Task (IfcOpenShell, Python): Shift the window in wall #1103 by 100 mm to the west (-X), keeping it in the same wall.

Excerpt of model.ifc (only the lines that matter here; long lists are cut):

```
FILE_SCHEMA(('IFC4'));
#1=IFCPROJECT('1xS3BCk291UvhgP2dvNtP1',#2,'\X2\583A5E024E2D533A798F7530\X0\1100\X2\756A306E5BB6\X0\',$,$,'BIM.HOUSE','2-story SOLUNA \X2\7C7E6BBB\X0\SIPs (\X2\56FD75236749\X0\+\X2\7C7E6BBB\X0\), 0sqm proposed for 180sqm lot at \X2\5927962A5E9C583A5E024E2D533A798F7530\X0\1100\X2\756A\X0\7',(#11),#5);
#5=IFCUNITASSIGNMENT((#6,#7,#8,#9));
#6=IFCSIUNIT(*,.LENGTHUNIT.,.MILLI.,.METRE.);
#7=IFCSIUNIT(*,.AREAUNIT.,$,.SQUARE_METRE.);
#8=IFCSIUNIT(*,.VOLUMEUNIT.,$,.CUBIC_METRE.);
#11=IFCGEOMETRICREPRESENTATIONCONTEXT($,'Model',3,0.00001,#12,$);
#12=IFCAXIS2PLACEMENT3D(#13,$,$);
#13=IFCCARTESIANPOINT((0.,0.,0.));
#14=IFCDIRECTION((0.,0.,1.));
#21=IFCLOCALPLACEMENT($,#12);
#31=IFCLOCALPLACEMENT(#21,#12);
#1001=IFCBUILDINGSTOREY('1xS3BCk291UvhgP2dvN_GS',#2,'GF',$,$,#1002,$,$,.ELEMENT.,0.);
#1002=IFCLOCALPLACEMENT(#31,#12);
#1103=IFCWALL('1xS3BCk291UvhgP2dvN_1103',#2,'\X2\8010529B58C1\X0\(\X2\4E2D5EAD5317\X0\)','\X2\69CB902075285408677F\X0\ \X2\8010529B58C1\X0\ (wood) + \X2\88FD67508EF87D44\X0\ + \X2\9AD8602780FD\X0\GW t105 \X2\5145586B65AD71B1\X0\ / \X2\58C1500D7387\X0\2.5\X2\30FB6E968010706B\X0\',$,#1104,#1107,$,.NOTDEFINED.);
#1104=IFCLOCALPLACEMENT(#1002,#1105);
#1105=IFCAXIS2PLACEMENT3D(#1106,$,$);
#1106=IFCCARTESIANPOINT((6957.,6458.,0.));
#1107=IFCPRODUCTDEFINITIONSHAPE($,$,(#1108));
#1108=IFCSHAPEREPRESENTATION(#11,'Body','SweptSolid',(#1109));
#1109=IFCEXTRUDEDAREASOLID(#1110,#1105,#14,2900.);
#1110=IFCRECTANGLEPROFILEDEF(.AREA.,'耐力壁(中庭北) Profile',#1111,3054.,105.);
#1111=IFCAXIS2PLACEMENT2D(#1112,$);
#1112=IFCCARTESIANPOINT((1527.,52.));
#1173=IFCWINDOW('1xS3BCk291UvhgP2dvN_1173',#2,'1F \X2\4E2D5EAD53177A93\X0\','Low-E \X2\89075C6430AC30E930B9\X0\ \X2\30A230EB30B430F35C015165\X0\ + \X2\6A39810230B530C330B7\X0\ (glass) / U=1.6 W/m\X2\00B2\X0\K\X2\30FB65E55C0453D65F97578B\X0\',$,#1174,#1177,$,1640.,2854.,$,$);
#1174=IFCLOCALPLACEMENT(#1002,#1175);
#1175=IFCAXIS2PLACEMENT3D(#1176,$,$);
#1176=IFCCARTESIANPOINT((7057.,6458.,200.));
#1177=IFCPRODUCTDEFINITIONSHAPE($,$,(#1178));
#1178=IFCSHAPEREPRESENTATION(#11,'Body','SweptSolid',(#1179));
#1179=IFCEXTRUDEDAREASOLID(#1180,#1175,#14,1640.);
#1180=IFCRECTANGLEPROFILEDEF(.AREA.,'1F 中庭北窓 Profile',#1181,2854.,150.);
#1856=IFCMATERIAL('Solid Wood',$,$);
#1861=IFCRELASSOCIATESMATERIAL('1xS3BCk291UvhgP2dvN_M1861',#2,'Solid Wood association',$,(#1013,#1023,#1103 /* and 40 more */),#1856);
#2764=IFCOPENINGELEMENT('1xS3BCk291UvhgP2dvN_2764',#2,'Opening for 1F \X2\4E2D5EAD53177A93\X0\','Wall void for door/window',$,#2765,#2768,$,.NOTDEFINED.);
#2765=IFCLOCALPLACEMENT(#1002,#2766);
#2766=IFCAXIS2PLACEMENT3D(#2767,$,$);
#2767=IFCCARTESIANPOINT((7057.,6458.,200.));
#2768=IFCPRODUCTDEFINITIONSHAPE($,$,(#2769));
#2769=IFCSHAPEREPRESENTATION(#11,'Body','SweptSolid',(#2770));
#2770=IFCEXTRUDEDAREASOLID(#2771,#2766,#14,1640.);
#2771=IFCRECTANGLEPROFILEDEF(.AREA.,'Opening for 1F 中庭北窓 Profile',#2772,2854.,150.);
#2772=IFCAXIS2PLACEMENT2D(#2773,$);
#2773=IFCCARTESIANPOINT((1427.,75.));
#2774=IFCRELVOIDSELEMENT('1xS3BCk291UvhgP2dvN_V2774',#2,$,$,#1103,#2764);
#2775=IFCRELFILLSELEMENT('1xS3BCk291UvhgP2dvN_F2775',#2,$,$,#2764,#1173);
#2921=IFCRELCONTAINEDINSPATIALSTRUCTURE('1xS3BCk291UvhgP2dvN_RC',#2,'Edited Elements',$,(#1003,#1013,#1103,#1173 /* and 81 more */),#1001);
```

```python
import ifcopenshell
import ifcopenshell.api.geometry
import ifcopenshell.util.placement
import ifcopenshell.util.unit

model = ifcopenshell.open("model.ifc")
unit_scale = ifcopenshell.util.unit.calculate_unit_scale(model)

window = model.by_guid("1xS3BCk291UvhgP2dvN_1173")
opening = window.FillsVoids[0].RelatingOpeningElement
wall = opening.VoidsElements[0].RelatingBuildingElement

wall_matrix = ifcopenshell.util.placement.get_local_placement(wall.ObjectPlacement)
shift = wall_matrix[:3, 0] * -0.1 / unit_scale
before = ifcopenshell.util.placement.get_local_placement(window.ObjectPlacement)[:3, 3].copy()

# The window is not placed relative to its opening, so move both.
for product in (opening, window):
    matrix = ifcopenshell.util.placement.get_local_placement(product.ObjectPlacement)
    matrix[:3, 3] += shift
    ifcopenshell.api.geometry.edit_object_placement(model, product=product, matrix=matrix, is_si=False)

after = ifcopenshell.util.placement.get_local_placement(window.ObjectPlacement)[:3, 3]
print("window moved by", (after - before).round(3) + 0.0)

model.write("model_rev.ifc")
```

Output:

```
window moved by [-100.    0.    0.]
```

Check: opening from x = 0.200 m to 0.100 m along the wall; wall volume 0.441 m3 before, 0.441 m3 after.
